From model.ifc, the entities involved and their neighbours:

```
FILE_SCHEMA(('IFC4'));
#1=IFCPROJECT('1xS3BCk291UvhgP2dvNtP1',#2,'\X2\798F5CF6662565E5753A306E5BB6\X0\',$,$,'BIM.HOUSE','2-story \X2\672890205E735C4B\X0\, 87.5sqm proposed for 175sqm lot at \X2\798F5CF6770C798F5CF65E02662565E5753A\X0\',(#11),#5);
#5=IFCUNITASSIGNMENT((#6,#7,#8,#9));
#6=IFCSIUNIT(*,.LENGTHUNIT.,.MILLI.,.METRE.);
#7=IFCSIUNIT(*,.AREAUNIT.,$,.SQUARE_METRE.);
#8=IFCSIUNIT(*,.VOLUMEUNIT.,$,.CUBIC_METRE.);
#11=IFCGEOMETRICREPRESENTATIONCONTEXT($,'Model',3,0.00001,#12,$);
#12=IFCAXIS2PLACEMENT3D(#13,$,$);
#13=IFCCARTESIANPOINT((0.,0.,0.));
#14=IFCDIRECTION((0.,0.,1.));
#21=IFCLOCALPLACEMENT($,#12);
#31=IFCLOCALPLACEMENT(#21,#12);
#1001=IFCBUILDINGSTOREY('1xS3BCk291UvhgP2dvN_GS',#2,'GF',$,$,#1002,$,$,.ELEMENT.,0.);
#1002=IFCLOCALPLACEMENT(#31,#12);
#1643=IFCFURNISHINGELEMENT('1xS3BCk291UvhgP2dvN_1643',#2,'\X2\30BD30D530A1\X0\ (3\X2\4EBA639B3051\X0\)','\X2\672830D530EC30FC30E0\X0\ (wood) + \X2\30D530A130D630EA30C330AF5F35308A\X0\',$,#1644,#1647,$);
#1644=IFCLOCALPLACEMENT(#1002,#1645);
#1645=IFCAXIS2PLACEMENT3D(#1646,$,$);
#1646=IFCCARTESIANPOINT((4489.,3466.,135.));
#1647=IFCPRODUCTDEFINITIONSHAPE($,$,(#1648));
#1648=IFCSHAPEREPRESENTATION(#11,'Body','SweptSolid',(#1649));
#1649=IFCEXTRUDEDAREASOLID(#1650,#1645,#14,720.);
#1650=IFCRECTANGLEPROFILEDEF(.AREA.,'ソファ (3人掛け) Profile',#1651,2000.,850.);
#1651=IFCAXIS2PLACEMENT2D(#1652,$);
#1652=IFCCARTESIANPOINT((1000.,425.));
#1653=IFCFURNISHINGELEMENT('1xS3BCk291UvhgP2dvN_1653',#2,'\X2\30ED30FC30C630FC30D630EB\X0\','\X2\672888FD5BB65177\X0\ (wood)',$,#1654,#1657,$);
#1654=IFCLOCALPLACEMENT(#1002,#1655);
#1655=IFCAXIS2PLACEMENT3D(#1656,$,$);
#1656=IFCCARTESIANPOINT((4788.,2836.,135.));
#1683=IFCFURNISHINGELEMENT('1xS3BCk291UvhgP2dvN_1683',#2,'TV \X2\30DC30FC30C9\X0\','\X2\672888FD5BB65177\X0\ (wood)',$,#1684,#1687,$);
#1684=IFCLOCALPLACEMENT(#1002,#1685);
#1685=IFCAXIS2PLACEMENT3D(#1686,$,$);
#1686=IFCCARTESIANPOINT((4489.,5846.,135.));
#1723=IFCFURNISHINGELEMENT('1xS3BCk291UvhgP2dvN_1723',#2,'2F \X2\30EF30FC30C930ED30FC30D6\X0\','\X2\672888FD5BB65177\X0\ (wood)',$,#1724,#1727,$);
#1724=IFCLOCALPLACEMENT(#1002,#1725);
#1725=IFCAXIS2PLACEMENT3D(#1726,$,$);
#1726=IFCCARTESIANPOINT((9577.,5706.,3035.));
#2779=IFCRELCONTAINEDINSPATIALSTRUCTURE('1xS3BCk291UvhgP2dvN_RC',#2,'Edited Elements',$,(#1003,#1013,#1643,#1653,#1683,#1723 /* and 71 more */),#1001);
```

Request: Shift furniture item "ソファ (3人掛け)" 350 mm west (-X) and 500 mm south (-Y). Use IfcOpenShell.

```python
import ifcopenshell
import ifcopenshell.api.geometry
import ifcopenshell.util.placement
import ifcopenshell.util.unit

model = ifcopenshell.open("model.ifc")
unit_scale = ifcopenshell.util.unit.calculate_unit_scale(model)

item = model.by_guid("1xS3BCk291UvhgP2dvN_1643")
matrix = ifcopenshell.util.placement.get_local_placement(item.ObjectPlacement)
matrix[0, 3] -= 0.35 / unit_scale
matrix[1, 3] -= 0.5 / unit_scale
ifcopenshell.api.geometry.edit_object_placement(model, product=item, matrix=matrix, is_si=False)

print(ifcopenshell.util.placement.get_local_placement(item.ObjectPlacement).round(3) + 0.0)

model.write("model_updated.ifc")
```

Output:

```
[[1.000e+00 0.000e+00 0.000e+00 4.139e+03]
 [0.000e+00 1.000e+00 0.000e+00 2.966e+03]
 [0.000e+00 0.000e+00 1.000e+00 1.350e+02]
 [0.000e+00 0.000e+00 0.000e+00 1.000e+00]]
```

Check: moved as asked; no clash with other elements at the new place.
